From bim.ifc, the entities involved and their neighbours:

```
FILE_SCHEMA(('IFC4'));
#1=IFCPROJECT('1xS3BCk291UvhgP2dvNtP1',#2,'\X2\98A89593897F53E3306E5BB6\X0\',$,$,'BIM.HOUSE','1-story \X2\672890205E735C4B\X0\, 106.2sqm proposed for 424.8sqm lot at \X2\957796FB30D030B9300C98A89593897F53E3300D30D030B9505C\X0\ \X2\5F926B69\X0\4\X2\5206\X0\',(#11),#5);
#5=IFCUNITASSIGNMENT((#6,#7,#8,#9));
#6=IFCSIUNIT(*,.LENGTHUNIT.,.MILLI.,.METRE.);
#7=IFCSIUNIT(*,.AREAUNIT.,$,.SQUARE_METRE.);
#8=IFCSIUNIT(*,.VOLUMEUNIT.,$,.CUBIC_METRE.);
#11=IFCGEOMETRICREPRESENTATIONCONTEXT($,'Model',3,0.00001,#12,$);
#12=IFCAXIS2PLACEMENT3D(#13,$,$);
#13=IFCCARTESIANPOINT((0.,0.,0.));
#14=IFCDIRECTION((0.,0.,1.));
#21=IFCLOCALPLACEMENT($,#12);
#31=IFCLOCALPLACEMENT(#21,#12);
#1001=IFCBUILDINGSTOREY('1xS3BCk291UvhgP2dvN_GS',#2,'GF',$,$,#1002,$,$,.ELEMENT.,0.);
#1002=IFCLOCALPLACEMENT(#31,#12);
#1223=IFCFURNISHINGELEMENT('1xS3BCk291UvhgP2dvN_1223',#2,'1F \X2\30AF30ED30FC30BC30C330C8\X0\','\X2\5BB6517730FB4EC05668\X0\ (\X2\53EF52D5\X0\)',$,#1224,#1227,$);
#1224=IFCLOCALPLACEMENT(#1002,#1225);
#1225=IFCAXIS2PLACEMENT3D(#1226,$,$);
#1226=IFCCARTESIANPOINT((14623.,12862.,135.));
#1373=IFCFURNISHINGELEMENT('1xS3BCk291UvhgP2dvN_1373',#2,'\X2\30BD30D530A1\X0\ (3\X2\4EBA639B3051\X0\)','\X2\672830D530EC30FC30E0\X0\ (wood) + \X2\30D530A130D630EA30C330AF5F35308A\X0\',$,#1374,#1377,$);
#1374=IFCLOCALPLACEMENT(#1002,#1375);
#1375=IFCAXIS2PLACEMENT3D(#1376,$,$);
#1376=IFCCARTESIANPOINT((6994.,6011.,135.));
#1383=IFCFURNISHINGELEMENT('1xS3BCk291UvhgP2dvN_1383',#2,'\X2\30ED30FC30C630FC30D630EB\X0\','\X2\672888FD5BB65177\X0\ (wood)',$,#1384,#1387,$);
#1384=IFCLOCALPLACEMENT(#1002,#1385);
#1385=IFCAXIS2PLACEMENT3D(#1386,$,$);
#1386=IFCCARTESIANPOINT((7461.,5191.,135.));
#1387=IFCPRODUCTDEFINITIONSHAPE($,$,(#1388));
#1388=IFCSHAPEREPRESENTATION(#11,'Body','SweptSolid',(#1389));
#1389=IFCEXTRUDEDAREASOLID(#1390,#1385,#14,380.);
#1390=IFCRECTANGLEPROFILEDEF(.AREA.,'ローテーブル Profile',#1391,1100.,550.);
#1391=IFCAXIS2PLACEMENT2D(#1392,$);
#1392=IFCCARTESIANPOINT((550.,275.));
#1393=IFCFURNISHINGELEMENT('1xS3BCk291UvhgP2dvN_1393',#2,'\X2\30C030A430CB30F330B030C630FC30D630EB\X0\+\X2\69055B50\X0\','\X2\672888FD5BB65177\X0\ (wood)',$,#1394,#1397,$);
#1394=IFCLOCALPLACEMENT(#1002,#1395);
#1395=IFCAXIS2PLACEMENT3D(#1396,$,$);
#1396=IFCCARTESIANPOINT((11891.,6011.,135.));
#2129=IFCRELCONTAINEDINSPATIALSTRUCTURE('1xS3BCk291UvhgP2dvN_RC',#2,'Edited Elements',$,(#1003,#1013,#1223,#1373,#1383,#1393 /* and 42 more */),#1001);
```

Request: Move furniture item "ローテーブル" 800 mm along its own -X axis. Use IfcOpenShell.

```python
import ifcopenshell
import ifcopenshell.api.geometry
import ifcopenshell.util.placement
import ifcopenshell.util.unit

model = ifcopenshell.open("bim.ifc")
unit_scale = ifcopenshell.util.unit.calculate_unit_scale(model)

item = model.by_id(1383)
matrix = ifcopenshell.util.placement.get_local_placement(item.ObjectPlacement)
matrix[:3, 3] -= matrix[:3, 0] * 0.8 / unit_scale
ifcopenshell.api.geometry.edit_object_placement(model, product=item, matrix=matrix, is_si=False)

print(ifcopenshell.util.placement.get_local_placement(item.ObjectPlacement).round(3) + 0.0)

model.write("bim_edited.ifc")
```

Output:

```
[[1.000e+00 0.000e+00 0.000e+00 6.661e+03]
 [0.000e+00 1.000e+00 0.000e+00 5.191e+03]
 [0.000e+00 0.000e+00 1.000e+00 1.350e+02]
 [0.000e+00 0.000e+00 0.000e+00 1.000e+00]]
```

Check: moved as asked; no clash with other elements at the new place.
